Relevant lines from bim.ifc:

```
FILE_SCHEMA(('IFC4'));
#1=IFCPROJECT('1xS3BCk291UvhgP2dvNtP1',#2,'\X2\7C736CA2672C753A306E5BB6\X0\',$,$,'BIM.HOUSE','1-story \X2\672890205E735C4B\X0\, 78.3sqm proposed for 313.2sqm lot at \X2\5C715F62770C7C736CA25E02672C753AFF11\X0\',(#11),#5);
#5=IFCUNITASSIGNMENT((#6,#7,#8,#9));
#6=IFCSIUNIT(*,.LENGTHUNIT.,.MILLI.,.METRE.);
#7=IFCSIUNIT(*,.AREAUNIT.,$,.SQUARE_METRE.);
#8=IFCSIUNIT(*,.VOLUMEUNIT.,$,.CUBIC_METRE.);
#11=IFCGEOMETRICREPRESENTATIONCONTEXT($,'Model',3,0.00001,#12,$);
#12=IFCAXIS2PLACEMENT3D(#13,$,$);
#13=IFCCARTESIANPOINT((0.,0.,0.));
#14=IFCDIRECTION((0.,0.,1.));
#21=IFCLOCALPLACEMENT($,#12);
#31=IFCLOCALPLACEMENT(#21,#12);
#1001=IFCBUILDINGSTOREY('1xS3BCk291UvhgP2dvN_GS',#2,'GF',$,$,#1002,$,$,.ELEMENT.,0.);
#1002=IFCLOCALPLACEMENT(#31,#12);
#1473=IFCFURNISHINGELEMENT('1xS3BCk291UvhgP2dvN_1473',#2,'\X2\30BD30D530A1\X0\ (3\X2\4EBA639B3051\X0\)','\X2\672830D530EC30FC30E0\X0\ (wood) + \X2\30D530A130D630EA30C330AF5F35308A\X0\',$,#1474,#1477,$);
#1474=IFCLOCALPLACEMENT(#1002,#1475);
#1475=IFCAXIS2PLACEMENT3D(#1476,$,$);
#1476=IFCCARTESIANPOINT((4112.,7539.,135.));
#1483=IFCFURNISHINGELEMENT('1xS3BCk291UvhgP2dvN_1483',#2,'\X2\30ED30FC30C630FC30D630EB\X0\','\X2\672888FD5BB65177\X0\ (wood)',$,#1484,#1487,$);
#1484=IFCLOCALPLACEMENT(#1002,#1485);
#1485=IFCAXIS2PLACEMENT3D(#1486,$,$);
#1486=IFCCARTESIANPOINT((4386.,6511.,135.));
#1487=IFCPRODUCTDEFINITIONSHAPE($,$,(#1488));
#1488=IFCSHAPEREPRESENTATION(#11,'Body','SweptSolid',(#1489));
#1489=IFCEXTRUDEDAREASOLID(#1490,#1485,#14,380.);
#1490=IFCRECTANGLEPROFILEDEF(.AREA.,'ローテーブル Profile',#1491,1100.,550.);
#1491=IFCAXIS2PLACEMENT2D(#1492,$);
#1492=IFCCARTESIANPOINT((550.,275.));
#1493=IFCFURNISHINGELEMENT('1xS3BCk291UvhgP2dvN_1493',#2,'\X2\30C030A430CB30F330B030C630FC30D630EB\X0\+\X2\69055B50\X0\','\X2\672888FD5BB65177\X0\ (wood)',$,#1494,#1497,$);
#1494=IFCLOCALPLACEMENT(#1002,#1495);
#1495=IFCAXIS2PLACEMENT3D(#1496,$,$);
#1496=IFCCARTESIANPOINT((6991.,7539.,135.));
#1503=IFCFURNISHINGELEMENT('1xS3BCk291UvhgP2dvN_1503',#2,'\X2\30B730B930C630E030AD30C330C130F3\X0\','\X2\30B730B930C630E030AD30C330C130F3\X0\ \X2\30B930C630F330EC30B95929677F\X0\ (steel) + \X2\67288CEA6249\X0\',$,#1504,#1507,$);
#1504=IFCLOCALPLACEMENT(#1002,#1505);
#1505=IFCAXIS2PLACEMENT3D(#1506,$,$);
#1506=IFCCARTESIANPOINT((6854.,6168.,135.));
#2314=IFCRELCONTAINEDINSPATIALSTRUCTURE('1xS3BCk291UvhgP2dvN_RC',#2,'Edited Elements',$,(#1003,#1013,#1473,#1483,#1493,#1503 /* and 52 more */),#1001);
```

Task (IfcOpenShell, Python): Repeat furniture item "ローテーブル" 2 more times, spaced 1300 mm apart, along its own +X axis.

```python
import ifcopenshell
import ifcopenshell.api.geometry
import ifcopenshell.api.root
import ifcopenshell.util.element
import ifcopenshell.util.placement

model = ifcopenshell.open("bim.ifc")


def reuse_history(source, copy):
    """copy_class also copies each property set's owner history, people and application; keep the originals."""
    for rel in copy.IsDefinedBy:
        if rel.is_a("IfcRelDefinesByProperties") and (history := rel.RelatingPropertyDefinition.OwnerHistory):
            rel.RelatingPropertyDefinition.OwnerHistory = source.OwnerHistory
            ifcopenshell.util.element.remove_deep2(model, history)


source = model.by_guid("1xS3BCk291UvhgP2dvN_1483")
base = ifcopenshell.util.placement.get_local_placement(source.ObjectPlacement)
step = base[:3, 0] * 1300.0

for i in range(1, 3):
    copy = ifcopenshell.api.root.copy_class(model, product=source)
    copy.Representation = ifcopenshell.util.element.copy_deep(
        model, source.Representation, exclude=["IfcGeometricRepresentationContext", "IfcRepresentationMap"]
    )
    reuse_history(source, copy)
    matrix = base.copy()
    matrix[:3, 3] += i * step
    print("added at", matrix[:3, 3].round(3) + 0.0)
    ifcopenshell.api.geometry.edit_object_placement(model, product=copy, matrix=matrix, is_si=False)

model.write("bim-out.ifc")
```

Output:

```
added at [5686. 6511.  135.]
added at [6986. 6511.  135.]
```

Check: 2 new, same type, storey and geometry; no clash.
